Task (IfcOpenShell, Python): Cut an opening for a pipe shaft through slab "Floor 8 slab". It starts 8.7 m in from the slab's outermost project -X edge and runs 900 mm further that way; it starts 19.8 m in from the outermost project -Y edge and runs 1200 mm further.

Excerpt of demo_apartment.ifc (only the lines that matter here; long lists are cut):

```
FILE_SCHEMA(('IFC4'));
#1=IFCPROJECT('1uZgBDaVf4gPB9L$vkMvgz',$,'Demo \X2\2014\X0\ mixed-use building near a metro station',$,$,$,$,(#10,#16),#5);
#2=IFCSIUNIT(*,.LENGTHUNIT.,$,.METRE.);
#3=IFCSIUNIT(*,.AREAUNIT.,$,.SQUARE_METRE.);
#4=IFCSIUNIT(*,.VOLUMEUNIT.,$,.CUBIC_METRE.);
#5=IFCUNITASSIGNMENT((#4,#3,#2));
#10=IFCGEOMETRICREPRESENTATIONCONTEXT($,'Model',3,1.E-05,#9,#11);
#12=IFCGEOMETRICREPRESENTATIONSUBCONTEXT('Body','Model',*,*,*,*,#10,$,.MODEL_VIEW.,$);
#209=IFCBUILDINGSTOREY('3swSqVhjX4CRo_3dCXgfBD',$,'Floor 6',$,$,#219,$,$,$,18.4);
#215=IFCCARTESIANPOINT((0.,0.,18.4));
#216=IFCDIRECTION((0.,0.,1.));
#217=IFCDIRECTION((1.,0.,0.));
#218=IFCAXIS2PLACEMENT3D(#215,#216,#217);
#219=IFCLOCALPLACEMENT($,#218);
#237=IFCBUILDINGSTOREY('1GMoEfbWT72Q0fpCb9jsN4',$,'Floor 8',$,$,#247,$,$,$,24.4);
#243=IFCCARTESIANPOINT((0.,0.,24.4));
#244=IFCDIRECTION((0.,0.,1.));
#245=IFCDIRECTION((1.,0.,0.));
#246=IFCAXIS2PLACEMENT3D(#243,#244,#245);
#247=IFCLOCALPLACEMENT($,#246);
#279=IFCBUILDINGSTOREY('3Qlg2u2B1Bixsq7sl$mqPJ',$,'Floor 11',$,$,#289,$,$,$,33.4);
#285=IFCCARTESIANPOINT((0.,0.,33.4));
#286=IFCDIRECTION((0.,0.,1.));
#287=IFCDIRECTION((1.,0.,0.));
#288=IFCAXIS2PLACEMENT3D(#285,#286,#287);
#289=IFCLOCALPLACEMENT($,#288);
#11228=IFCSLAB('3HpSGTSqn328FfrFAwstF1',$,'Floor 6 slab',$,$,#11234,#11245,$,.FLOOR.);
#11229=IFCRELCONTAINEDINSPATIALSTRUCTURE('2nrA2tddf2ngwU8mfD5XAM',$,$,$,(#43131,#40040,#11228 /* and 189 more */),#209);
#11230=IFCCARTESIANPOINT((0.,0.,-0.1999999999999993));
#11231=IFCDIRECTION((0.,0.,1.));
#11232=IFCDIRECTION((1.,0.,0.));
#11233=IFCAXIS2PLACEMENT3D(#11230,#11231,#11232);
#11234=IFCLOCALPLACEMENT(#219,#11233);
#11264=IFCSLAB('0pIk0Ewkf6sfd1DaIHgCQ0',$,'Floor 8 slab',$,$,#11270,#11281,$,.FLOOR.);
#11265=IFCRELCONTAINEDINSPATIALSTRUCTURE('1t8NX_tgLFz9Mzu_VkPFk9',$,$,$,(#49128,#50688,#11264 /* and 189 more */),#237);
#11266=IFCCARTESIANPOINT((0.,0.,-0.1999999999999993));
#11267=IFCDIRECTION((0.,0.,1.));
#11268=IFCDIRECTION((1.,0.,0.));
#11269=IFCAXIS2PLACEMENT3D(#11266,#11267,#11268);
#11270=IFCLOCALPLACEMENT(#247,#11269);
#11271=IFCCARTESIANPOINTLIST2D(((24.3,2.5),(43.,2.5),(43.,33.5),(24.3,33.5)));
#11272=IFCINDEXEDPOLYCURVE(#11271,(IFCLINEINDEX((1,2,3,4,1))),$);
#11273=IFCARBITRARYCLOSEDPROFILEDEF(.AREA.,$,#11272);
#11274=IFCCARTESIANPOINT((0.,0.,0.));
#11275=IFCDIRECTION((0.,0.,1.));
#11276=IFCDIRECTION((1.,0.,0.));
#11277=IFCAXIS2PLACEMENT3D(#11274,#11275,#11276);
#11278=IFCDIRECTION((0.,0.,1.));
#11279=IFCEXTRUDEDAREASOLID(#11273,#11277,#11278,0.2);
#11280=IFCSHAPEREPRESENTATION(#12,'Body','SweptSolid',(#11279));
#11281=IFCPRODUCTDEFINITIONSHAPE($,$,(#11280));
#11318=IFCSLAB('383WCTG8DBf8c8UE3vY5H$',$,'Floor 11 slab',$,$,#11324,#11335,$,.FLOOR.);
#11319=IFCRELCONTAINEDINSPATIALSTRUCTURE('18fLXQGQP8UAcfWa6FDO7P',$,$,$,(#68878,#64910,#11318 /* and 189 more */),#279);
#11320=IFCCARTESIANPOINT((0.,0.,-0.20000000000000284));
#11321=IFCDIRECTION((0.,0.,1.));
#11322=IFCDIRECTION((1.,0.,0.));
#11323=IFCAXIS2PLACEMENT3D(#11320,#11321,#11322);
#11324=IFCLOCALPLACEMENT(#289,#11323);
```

```python
import numpy as np
import ifcopenshell
import ifcopenshell.api.feature
import ifcopenshell.api.geometry
import ifcopenshell.api.root
import ifcopenshell.geom
import ifcopenshell.util.placement
import ifcopenshell.util.representation
import ifcopenshell.util.shape
import ifcopenshell.util.unit

model = ifcopenshell.open("demo_apartment.ifc")
unit_scale = ifcopenshell.util.unit.calculate_unit_scale(model)
settings = ifcopenshell.geom.settings()


def volume(element):
    """Net volume in cubic metres, openings subtracted."""
    shape = ifcopenshell.geom.create_shape(settings, element)
    return ifcopenshell.util.shape.get_volume(shape.geometry)


slab = model.by_guid("0pIk0Ewkf6sfd1DaIHgCQ0")
before = volume(slab)

# Extent in the slab's own axes, in metres. The edges named are its -X and -Y sides.
slab_shape = ifcopenshell.geom.create_shape(settings, slab)
vertices = ifcopenshell.util.shape.get_vertices(slab_shape.geometry)
x_min, y_min, bottom = vertices.min(axis=0)
top = vertices[:, 2].max()

opening = ifcopenshell.api.root.create_entity(model, ifc_class="IfcOpeningElement", name="Pipe shaft opening", predefined_type="OPENING")
context = ifcopenshell.util.representation.get_context(model, "Model", "Body", "MODEL_VIEW")
width, depth = 0.9, 1.2
outline = [(0.0, 0.0), (width, 0.0), (width, depth), (0.0, depth), (0.0, 0.0)]
# Overshoot both faces by 50 mm so the cut is clean.
shape = ifcopenshell.api.geometry.add_slab_representation(
    model, context=context, depth=top - bottom + 0.1, polyline=outline
)
ifcopenshell.api.geometry.assign_representation(model, product=opening, representation=shape)

matrix = ifcopenshell.util.placement.get_local_placement(slab.ObjectPlacement)
matrix[:, 3] = matrix @ np.append(np.array([x_min + 8.7, y_min + 19.8, bottom - 0.05]) / unit_scale, 1.0)
ifcopenshell.api.geometry.edit_object_placement(model, product=opening, matrix=matrix, is_si=False)
ifcopenshell.api.feature.add_feature(model, feature=opening, element=slab)

after = volume(slab)

print(f"slab volume {before:.3f} -> {after:.3f} m3")

model.write("demo_apartment_rev.ifc")
```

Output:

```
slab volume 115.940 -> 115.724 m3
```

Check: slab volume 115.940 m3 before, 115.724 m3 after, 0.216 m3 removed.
